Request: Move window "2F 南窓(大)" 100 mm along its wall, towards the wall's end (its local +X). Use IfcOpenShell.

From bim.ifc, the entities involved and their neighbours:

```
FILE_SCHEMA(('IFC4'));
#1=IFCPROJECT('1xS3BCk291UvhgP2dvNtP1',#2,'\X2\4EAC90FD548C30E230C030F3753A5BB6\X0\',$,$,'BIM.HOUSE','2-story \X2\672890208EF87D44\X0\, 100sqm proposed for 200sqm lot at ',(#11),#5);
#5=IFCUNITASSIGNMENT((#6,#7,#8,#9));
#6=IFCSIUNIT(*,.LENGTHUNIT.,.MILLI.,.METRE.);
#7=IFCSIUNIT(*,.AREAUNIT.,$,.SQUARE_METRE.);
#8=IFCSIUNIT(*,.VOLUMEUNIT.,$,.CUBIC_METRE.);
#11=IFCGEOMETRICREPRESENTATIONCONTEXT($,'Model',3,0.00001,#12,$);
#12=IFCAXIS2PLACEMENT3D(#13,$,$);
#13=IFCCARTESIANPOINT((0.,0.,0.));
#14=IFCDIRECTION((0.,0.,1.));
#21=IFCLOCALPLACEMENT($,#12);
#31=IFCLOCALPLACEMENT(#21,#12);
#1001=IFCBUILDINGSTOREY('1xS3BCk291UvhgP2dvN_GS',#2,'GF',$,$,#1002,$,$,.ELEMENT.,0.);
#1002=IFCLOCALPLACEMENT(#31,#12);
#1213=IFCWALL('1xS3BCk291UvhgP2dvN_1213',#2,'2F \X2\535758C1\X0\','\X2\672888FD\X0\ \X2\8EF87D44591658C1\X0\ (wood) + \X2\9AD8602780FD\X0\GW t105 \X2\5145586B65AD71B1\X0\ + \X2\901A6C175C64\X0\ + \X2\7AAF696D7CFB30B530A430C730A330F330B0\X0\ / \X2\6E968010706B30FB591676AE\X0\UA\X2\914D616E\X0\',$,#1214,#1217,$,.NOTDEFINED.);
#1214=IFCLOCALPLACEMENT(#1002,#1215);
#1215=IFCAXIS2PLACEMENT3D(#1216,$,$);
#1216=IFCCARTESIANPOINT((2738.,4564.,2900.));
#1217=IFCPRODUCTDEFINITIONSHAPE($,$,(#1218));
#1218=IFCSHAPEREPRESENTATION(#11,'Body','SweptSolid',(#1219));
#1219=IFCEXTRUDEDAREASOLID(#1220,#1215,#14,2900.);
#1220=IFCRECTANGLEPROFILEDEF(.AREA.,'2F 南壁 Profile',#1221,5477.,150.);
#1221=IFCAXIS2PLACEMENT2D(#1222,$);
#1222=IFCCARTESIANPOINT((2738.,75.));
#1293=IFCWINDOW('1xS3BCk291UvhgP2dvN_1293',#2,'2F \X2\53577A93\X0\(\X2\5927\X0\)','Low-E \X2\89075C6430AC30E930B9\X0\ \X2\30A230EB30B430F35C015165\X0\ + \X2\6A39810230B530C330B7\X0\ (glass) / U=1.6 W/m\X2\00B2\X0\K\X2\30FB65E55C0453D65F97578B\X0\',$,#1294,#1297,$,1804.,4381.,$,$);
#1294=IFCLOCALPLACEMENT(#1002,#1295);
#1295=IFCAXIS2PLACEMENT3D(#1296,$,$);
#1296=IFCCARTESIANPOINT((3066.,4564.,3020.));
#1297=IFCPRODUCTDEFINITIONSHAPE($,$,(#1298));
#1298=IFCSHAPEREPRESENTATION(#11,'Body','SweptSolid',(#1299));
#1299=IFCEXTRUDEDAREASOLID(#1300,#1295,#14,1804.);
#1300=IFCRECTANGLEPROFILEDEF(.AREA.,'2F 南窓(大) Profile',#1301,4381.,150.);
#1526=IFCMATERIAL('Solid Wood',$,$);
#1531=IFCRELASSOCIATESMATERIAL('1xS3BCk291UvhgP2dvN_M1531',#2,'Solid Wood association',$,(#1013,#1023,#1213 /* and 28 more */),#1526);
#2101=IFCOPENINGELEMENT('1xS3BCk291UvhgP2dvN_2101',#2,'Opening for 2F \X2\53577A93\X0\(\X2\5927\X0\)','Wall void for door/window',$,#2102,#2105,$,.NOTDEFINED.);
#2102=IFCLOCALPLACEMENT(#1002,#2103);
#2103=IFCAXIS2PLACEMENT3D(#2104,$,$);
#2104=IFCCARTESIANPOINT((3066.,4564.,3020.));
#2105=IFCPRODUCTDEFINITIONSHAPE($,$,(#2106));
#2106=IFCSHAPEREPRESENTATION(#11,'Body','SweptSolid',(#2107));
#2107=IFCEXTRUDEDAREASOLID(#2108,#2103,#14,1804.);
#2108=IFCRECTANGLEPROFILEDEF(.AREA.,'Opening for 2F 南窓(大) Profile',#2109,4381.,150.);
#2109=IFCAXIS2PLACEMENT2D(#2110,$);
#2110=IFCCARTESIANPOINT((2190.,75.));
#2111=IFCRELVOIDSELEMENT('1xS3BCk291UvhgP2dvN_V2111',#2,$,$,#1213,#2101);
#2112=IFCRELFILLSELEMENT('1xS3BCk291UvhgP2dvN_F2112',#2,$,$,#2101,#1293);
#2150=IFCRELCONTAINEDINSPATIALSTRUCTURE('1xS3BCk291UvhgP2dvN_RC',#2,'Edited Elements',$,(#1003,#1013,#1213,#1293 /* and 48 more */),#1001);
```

```python
import ifcopenshell
import ifcopenshell.api.geometry
import ifcopenshell.util.placement

model = ifcopenshell.open("bim.ifc")

window = model.by_guid("1xS3BCk291UvhgP2dvN_1293")
opening = window.FillsVoids[0].RelatingOpeningElement
wall = opening.VoidsElements[0].RelatingBuildingElement

wall_matrix = ifcopenshell.util.placement.get_local_placement(wall.ObjectPlacement)
shift = wall_matrix[:3, 0] * 100.0
before = ifcopenshell.util.placement.get_local_placement(window.ObjectPlacement)[:3, 3].copy()

# The window is not placed relative to its opening, so move both.
for product in (opening, window):
    matrix = ifcopenshell.util.placement.get_local_placement(product.ObjectPlacement)
    matrix[:3, 3] += shift
    ifcopenshell.api.geometry.edit_object_placement(model, product=product, matrix=matrix, is_si=False)

after = ifcopenshell.util.placement.get_local_placement(window.ObjectPlacement)[:3, 3]
print("window moved by", (after - before).round(3) + 0.0)

model.write("bim_edited.ifc")
```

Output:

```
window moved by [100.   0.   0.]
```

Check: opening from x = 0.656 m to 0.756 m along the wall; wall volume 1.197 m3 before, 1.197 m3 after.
